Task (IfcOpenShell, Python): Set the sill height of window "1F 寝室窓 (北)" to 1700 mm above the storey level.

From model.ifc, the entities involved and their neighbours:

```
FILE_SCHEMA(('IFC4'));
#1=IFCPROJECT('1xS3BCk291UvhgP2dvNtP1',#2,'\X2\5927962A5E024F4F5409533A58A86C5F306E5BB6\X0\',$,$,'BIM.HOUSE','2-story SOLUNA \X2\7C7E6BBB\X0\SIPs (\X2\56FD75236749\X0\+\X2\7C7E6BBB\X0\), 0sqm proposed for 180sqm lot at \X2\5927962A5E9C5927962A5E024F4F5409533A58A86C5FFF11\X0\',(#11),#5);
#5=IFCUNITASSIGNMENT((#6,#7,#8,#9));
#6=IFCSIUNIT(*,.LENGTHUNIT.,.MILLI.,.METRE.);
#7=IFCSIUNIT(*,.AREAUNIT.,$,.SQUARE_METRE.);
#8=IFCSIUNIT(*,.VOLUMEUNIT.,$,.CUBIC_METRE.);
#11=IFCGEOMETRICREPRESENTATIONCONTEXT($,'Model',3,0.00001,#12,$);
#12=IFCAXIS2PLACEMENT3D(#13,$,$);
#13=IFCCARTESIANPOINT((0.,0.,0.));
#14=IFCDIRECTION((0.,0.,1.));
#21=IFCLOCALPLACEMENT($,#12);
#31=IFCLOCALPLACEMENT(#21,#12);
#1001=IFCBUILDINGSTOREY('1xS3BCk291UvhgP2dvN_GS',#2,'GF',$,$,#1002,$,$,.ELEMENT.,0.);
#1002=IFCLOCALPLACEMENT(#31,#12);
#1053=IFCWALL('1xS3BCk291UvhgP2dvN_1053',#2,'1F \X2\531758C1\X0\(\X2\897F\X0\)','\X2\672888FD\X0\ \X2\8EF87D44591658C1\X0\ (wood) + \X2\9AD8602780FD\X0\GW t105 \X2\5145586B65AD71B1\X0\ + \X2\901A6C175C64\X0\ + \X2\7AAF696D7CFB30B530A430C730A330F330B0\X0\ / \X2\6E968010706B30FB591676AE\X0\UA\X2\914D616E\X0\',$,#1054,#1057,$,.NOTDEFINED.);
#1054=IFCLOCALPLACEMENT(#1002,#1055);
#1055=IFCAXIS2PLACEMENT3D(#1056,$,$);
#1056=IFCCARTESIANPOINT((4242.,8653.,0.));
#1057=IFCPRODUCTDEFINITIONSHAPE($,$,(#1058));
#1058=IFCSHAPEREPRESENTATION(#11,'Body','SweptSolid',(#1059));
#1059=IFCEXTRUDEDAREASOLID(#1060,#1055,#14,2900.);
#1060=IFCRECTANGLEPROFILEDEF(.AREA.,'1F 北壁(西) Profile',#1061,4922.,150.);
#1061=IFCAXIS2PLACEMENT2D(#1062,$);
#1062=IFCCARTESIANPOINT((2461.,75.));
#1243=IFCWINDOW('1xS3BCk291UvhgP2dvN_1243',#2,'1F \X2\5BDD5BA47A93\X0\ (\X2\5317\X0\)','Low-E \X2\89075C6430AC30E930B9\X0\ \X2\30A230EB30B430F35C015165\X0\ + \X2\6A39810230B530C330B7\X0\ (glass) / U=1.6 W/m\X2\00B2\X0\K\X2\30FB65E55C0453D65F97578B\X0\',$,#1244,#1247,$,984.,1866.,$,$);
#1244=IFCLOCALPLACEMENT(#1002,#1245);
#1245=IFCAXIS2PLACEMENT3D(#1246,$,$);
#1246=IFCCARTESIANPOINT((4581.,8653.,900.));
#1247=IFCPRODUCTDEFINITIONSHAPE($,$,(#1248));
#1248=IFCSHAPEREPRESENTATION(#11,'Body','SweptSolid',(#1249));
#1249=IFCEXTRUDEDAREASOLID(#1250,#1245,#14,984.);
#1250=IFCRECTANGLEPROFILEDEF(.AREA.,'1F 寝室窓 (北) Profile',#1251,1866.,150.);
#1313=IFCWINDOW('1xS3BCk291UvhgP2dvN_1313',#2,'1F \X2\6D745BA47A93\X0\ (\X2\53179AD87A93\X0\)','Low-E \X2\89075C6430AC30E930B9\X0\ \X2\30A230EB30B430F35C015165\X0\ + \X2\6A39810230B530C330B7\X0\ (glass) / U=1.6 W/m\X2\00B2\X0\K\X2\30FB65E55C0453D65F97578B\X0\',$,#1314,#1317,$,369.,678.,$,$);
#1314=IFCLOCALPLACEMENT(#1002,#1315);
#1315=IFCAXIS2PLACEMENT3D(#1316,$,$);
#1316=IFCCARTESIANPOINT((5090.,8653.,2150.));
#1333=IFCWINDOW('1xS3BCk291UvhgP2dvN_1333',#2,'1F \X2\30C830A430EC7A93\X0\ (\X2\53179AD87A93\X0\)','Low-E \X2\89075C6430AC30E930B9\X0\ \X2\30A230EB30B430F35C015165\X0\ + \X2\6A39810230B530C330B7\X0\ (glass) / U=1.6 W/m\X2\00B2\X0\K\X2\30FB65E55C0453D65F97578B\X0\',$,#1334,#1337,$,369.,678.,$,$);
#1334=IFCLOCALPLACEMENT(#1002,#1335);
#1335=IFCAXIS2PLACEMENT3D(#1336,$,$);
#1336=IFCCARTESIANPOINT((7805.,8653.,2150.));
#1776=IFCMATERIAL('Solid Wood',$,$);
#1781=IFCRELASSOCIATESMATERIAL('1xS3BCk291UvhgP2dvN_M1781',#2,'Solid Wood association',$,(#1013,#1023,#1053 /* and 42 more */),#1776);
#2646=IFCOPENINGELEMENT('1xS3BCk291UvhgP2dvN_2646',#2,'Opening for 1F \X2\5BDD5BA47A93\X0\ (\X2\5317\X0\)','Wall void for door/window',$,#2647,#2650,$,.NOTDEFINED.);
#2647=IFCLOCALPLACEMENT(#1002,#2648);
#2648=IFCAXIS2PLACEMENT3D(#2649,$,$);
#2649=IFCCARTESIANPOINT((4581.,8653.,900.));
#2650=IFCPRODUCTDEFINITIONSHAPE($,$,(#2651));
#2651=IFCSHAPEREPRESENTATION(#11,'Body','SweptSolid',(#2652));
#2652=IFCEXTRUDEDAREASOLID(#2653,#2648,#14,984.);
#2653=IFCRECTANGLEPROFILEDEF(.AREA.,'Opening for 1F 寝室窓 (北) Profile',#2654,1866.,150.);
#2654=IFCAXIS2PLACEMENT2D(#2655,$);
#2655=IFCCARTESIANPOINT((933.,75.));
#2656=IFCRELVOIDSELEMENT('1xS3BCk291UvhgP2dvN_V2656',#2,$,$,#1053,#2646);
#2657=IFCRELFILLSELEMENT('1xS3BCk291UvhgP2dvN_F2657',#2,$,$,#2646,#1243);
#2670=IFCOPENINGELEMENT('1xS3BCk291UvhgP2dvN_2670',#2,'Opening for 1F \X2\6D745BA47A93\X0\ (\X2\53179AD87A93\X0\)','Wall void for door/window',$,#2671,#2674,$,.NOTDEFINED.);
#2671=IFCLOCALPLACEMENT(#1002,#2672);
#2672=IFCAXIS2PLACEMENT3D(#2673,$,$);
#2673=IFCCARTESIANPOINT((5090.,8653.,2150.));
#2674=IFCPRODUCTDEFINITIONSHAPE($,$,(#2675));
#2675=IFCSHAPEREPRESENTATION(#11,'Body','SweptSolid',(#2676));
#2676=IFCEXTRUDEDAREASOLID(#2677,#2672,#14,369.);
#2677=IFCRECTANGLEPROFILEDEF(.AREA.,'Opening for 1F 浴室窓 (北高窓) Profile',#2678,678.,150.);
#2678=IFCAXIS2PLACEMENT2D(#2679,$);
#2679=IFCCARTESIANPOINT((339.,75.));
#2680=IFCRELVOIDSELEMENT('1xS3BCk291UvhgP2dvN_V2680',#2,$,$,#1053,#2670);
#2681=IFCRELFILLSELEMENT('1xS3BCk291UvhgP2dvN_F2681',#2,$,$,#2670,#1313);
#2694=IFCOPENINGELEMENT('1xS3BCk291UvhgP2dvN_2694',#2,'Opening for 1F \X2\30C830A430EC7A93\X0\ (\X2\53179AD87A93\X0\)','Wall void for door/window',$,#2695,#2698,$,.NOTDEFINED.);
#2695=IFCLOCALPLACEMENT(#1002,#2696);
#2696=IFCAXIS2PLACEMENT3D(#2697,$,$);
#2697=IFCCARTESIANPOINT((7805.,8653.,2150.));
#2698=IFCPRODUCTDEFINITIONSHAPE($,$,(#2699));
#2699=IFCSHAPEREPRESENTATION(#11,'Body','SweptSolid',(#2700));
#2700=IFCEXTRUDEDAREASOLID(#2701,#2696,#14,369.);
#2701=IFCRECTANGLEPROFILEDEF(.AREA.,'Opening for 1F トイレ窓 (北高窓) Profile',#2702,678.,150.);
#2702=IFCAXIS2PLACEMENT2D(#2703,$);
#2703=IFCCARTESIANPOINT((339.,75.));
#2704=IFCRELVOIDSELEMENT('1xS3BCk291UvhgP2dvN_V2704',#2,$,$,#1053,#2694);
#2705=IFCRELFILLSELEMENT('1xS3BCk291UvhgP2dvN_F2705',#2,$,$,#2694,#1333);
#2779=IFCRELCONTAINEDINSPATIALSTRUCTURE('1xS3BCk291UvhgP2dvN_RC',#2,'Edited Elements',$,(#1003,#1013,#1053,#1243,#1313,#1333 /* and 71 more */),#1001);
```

```python
import numpy as np
import ifcopenshell
import ifcopenshell.api.geometry
import ifcopenshell.geom
import ifcopenshell.util.element
import ifcopenshell.util.placement
import ifcopenshell.util.shape
import ifcopenshell.util.unit

model = ifcopenshell.open("model.ifc")
unit_scale = ifcopenshell.util.unit.calculate_unit_scale(model)

window = model.by_guid("1xS3BCk291UvhgP2dvN_1243")
opening = window.FillsVoids[0].RelatingOpeningElement
storey = ifcopenshell.util.element.get_container(window, ifc_class="IfcBuildingStorey")
level = ifcopenshell.util.placement.get_local_placement(storey.ObjectPlacement)[2, 3]

# The opening's origin need not be at the sill, so measure its lowest point.
shape = ifcopenshell.geom.create_shape(ifcopenshell.geom.settings(), opening)
bottom = ifcopenshell.util.shape.get_shape_bottom_elevation(shape, shape.geometry) / unit_scale
dz = level + 1.7 / unit_scale - bottom

shift = np.array([0.0, 0.0, dz])
# The window is not placed relative to its opening, so move both.
for product in (opening, window):
    matrix = ifcopenshell.util.placement.get_local_placement(product.ObjectPlacement)
    matrix[:3, 3] += shift
    ifcopenshell.api.geometry.edit_object_placement(model, product=product, matrix=matrix, is_si=False)

print(f"moved by {dz * unit_scale:+.3f} m")

model.write("model_edited.ifc")
```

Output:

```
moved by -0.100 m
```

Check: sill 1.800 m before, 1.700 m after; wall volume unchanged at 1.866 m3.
